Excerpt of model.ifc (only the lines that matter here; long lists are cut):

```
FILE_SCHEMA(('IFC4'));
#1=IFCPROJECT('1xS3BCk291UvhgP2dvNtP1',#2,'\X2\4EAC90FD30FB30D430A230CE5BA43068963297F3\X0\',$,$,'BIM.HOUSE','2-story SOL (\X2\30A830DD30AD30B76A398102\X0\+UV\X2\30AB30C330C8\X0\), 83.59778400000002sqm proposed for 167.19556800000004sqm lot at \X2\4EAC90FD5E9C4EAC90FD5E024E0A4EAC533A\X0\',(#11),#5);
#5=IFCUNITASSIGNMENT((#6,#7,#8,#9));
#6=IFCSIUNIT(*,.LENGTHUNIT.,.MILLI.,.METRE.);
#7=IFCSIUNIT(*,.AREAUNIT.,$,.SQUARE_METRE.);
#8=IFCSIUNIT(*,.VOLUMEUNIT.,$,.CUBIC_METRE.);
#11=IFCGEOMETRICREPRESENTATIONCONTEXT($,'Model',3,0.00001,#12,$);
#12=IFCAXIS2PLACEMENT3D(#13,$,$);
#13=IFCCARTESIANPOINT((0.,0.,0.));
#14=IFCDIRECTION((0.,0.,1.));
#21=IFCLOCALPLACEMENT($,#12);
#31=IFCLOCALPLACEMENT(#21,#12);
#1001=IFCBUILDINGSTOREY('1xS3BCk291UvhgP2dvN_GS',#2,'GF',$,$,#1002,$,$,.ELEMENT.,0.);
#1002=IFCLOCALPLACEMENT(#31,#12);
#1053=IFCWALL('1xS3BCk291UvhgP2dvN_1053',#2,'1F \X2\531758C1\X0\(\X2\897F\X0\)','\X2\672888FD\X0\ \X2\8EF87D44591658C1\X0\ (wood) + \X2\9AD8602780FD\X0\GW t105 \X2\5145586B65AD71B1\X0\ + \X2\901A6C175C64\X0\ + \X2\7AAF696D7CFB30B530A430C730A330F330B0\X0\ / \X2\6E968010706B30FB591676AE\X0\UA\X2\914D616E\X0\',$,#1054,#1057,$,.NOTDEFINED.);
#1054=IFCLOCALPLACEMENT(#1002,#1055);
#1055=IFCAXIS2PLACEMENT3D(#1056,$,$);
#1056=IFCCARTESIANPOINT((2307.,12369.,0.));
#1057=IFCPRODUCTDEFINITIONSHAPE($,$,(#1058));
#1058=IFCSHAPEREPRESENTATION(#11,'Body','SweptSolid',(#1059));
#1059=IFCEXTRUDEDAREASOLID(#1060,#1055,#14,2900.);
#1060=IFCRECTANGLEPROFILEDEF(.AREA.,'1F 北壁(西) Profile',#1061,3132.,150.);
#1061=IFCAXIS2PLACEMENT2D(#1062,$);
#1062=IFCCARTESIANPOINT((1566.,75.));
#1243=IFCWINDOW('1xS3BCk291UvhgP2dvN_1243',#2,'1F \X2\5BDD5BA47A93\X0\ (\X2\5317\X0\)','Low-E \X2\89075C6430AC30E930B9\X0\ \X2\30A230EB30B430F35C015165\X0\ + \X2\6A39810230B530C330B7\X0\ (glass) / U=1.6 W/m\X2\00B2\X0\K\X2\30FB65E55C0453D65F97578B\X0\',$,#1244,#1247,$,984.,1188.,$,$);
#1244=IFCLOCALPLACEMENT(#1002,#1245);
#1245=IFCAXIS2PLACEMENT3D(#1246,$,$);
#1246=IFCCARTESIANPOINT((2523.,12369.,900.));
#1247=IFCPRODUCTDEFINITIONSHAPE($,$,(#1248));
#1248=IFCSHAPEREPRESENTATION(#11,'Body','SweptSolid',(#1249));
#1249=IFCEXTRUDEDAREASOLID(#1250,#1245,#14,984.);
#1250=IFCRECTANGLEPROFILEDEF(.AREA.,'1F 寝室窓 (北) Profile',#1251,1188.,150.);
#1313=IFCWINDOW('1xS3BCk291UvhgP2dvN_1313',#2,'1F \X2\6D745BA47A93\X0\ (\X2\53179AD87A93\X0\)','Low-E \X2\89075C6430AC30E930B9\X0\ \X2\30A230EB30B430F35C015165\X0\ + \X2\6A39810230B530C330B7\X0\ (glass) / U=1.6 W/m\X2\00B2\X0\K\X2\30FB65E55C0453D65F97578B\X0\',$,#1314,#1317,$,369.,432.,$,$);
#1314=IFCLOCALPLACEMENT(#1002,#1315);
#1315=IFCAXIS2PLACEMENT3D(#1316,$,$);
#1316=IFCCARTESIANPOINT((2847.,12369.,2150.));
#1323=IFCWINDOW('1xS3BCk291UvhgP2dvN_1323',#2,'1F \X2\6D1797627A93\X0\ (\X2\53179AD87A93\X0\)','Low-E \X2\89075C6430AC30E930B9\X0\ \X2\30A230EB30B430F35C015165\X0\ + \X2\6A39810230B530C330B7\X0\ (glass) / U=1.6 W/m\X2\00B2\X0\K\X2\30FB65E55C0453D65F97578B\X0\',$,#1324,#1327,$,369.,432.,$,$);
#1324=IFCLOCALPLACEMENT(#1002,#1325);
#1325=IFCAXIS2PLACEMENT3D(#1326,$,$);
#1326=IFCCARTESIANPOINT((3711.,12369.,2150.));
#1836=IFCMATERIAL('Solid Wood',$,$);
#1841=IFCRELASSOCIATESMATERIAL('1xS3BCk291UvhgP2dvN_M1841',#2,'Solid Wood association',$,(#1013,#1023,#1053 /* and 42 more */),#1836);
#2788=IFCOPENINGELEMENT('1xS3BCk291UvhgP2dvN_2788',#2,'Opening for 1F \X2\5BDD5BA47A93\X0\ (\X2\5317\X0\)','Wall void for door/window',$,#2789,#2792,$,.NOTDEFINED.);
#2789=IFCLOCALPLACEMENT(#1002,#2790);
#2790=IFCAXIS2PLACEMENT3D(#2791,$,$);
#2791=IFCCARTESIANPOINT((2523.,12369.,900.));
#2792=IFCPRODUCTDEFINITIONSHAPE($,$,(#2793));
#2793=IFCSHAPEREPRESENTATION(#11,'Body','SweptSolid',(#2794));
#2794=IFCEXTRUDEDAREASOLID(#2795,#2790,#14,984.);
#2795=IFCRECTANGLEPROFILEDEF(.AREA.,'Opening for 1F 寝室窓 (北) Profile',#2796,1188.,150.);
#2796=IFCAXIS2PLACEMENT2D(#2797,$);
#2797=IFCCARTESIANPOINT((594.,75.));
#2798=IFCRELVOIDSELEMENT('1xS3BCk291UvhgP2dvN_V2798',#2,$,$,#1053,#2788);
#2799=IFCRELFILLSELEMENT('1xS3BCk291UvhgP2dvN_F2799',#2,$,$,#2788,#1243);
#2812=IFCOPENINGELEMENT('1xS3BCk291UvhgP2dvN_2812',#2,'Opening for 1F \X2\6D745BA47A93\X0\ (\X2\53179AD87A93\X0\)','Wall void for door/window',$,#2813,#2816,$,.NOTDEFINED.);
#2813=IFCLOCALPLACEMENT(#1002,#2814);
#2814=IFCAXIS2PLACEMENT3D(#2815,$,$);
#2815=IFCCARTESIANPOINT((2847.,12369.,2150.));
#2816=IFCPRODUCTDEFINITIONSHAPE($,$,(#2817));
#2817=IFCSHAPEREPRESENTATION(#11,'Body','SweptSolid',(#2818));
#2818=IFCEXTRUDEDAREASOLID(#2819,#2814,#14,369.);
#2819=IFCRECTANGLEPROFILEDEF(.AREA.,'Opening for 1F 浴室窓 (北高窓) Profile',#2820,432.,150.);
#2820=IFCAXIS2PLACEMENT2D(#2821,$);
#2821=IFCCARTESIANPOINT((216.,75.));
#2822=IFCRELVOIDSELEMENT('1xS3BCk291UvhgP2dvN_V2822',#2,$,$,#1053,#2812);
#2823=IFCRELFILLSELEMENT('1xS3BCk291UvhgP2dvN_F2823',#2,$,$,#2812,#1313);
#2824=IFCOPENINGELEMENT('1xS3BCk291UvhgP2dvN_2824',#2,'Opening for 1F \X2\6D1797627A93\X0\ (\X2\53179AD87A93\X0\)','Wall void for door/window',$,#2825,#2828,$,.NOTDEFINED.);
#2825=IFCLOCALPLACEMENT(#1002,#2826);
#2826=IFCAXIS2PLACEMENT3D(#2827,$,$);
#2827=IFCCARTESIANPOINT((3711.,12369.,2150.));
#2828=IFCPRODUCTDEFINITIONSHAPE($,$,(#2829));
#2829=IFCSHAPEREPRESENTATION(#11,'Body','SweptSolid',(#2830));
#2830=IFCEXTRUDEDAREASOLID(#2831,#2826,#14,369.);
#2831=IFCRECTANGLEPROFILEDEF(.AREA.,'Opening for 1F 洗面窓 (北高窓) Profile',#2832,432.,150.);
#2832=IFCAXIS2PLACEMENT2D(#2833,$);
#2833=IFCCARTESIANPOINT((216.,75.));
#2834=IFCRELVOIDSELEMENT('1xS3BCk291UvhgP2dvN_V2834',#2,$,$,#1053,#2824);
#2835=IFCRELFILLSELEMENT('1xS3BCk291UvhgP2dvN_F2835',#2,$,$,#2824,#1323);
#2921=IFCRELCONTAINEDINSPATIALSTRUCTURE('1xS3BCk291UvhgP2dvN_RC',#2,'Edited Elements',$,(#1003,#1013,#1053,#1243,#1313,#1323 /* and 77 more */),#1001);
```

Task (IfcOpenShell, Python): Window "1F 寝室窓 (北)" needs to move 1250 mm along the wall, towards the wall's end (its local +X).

```python
import ifcopenshell
import ifcopenshell.api.geometry
import ifcopenshell.util.placement
import ifcopenshell.util.unit

model = ifcopenshell.open("model.ifc")
unit_scale = ifcopenshell.util.unit.calculate_unit_scale(model)

window = model.by_guid("1xS3BCk291UvhgP2dvN_1243")
opening = window.FillsVoids[0].RelatingOpeningElement
wall = opening.VoidsElements[0].RelatingBuildingElement

wall_matrix = ifcopenshell.util.placement.get_local_placement(wall.ObjectPlacement)
shift = wall_matrix[:3, 0] * 1.25 / unit_scale
before = ifcopenshell.util.placement.get_local_placement(window.ObjectPlacement)[:3, 3].copy()

# The window is not placed relative to its opening, so move both.
for product in (opening, window):
    matrix = ifcopenshell.util.placement.get_local_placement(product.ObjectPlacement)
    matrix[:3, 3] += shift
    ifcopenshell.api.geometry.edit_object_placement(model, product=product, matrix=matrix, is_si=False)

after = ifcopenshell.util.placement.get_local_placement(window.ObjectPlacement)[:3, 3]
print("window moved by", (after - before).round(3) + 0.0)

model.write("model-out.ifc")
```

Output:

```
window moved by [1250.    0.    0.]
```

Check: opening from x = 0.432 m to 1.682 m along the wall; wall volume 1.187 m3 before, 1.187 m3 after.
